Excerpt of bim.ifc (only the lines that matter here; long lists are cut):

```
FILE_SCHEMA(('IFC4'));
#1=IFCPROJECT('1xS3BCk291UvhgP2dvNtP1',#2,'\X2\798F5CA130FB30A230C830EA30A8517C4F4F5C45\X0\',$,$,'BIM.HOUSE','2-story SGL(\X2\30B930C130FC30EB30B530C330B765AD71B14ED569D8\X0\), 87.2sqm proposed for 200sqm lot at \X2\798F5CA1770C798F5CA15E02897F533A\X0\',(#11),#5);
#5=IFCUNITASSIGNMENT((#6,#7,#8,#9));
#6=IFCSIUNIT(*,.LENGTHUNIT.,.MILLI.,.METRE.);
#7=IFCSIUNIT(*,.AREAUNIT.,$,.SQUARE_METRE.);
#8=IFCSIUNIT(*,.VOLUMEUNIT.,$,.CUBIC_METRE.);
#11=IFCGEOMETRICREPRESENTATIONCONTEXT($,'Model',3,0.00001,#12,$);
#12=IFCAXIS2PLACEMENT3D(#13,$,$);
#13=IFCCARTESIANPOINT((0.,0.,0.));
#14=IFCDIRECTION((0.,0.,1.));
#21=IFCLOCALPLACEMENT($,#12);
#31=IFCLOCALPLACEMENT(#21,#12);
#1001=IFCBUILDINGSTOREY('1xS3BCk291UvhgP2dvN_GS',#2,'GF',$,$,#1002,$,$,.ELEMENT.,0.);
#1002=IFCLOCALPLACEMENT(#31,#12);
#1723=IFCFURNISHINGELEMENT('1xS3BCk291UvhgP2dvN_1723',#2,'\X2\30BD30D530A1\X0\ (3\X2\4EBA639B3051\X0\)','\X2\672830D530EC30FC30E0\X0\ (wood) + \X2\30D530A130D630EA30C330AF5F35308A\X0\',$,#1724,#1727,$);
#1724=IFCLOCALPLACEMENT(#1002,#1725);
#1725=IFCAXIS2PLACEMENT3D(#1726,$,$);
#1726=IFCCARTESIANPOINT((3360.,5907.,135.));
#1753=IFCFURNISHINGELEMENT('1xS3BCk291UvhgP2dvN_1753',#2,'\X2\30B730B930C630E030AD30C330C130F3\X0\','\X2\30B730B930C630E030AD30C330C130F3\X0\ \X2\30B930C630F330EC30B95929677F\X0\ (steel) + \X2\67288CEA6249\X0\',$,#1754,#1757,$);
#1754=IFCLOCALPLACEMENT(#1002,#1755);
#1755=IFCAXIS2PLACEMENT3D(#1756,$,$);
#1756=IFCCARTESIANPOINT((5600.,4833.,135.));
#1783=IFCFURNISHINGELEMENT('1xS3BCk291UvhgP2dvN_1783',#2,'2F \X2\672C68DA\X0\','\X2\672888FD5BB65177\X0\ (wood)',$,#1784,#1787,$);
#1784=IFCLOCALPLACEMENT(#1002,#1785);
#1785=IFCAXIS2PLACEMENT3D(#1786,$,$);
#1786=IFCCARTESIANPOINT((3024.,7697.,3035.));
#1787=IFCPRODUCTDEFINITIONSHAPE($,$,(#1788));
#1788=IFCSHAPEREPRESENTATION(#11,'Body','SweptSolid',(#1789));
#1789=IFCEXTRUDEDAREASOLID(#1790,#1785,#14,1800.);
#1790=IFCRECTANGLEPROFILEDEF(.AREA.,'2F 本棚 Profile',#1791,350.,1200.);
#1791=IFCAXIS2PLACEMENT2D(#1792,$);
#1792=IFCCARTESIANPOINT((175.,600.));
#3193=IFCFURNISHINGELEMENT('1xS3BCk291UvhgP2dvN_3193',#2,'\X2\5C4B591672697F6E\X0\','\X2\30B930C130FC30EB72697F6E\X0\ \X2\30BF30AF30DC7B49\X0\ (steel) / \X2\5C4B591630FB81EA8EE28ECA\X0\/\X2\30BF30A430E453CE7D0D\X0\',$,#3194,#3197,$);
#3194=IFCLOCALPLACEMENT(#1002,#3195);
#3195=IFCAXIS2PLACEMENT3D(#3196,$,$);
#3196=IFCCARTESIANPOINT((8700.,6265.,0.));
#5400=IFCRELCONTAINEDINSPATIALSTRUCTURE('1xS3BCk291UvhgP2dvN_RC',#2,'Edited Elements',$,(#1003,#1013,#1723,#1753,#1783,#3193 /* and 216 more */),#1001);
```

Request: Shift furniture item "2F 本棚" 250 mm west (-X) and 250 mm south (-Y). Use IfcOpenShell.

```python
import ifcopenshell
import ifcopenshell.api.geometry
import ifcopenshell.util.placement

model = ifcopenshell.open("bim.ifc")

item = model.by_guid("1xS3BCk291UvhgP2dvN_1783")
matrix = ifcopenshell.util.placement.get_local_placement(item.ObjectPlacement)
matrix[0, 3] -= 250.0
matrix[1, 3] -= 250.0
ifcopenshell.api.geometry.edit_object_placement(model, product=item, matrix=matrix, is_si=False)

print(ifcopenshell.util.placement.get_local_placement(item.ObjectPlacement).round(3) + 0.0)

model.write("bim-out.ifc")
```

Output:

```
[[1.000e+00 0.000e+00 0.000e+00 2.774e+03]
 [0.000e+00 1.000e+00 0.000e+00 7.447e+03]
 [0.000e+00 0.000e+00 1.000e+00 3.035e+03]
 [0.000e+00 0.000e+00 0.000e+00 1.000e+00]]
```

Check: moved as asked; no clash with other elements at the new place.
